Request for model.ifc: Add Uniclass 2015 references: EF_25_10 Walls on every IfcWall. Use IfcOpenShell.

First a look at what the model holds.

```python
import ifcopenshell

model = ifcopenshell.open("model.ifc")
print(model.schema)
print("classifications:", [c.Name for c in model.by_type("IfcClassification")])
for ifc_class in ("IfcDoor", "IfcRoof", "IfcStair", "IfcWall", "IfcWindow"):
    print(ifc_class, len(model.by_type(ifc_class)))
```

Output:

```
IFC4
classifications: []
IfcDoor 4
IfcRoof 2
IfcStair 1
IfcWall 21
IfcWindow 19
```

```python
import ifcopenshell
import ifcopenshell.api.classification

model = ifcopenshell.open("model.ifc")

system = ifcopenshell.api.classification.add_classification(model, classification="Uniclass 2015")

codes = {
    "IfcWall": ("EF_25_10", "Walls"),
}
for ifc_class, (code, name) in codes.items():
    products = model.by_type(ifc_class)
    ifcopenshell.api.classification.add_reference(
        model, products=products, classification=system, identification=code, name=name
    )
    print(code, len(products))

model.write("model_updated.ifc")
```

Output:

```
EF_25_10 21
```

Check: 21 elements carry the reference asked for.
